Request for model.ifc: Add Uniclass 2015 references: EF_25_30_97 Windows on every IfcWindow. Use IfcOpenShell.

First a look at what the model holds.

```python
import ifcopenshell

model = ifcopenshell.open("model.ifc")
print(model.schema)
print("classifications:", [c.Name for c in model.by_type("IfcClassification")])
for ifc_class in ("IfcDoor", "IfcRoof", "IfcStair", "IfcWall", "IfcWindow"):
    print(ifc_class, len(model.by_type(ifc_class)))
```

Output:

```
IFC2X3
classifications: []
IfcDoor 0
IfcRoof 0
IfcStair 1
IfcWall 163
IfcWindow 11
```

```python
import ifcopenshell
import ifcopenshell.api.classification

model = ifcopenshell.open("model.ifc")

# IFC2X3 requires Source and Edition and has no link from the project to the system.
system = model.create_entity("IfcClassification", Source="NBS", Edition="2015", Name="Uniclass 2015")

codes = {
    "IfcWindow": ("EF_25_30_97", "Windows"),
}
for ifc_class, (code, name) in codes.items():
    products = model.by_type(ifc_class)
    ifcopenshell.api.classification.add_reference(
        model, products=products, classification=system, identification=code, name=name
    )
    print(code, len(products))

model.write("model_rev.ifc")
```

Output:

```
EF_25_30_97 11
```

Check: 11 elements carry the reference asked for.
